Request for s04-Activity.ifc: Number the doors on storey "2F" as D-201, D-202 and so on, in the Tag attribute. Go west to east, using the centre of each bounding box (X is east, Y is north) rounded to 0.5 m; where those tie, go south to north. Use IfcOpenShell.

First a look at what the model holds.

```python
import ifcopenshell
import ifcopenshell.util.element
import ifcopenshell.util.placement

model = ifcopenshell.open("s04-Activity.ifc")
print(model.schema)
storey = next(s for s in model.by_type("IfcBuildingStorey") if s.Name == "2F")
doors = [e for e in ifcopenshell.util.element.get_decomposition(storey) if e.is_a("IfcDoor")]
for e in sorted(doors, key=lambda e: e.id()):
    origin = ifcopenshell.util.placement.get_local_placement(e.ObjectPlacement)[:3, 3]
    print(e.id(), e.Tag, e.Name, origin.round(2) + 0.0, sep=" | ")
```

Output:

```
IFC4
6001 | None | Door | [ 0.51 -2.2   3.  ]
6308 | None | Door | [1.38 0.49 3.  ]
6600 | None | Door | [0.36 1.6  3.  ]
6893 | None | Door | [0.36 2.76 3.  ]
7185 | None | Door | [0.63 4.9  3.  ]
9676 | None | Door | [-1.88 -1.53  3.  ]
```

```python
import ifcopenshell
import ifcopenshell.geom
import ifcopenshell.util.element
import ifcopenshell.util.shape

model = ifcopenshell.open("s04-Activity.ifc")
settings = ifcopenshell.geom.settings()
settings.set("use-world-coords", True)


def centre(element):
    shape = ifcopenshell.geom.create_shape(settings, element)
    return ifcopenshell.util.shape.get_bbox_centroid(shape.geometry)


storey = next(s for s in model.by_type("IfcBuildingStorey") if s.Name == "2F")
doors = [e for e in ifcopenshell.util.element.get_decomposition(storey) if e.is_a("IfcDoor")]

# Insertion points can sit at a corner or the storey origin, so sort by the geometry (in metres).
centres = {e: centre(e) for e in doors}
doors.sort(key=lambda e: (round(centres[e][0] / 0.5), centres[e][1]))

for i, e in enumerate(doors, start=1):
    number = f"D-2{i:02d}"
    e.Tag = number
    print(e.id(), number)

model.write("s04-Activity_updated.ifc")
```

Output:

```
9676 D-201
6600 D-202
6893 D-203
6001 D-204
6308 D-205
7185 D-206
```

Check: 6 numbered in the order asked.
